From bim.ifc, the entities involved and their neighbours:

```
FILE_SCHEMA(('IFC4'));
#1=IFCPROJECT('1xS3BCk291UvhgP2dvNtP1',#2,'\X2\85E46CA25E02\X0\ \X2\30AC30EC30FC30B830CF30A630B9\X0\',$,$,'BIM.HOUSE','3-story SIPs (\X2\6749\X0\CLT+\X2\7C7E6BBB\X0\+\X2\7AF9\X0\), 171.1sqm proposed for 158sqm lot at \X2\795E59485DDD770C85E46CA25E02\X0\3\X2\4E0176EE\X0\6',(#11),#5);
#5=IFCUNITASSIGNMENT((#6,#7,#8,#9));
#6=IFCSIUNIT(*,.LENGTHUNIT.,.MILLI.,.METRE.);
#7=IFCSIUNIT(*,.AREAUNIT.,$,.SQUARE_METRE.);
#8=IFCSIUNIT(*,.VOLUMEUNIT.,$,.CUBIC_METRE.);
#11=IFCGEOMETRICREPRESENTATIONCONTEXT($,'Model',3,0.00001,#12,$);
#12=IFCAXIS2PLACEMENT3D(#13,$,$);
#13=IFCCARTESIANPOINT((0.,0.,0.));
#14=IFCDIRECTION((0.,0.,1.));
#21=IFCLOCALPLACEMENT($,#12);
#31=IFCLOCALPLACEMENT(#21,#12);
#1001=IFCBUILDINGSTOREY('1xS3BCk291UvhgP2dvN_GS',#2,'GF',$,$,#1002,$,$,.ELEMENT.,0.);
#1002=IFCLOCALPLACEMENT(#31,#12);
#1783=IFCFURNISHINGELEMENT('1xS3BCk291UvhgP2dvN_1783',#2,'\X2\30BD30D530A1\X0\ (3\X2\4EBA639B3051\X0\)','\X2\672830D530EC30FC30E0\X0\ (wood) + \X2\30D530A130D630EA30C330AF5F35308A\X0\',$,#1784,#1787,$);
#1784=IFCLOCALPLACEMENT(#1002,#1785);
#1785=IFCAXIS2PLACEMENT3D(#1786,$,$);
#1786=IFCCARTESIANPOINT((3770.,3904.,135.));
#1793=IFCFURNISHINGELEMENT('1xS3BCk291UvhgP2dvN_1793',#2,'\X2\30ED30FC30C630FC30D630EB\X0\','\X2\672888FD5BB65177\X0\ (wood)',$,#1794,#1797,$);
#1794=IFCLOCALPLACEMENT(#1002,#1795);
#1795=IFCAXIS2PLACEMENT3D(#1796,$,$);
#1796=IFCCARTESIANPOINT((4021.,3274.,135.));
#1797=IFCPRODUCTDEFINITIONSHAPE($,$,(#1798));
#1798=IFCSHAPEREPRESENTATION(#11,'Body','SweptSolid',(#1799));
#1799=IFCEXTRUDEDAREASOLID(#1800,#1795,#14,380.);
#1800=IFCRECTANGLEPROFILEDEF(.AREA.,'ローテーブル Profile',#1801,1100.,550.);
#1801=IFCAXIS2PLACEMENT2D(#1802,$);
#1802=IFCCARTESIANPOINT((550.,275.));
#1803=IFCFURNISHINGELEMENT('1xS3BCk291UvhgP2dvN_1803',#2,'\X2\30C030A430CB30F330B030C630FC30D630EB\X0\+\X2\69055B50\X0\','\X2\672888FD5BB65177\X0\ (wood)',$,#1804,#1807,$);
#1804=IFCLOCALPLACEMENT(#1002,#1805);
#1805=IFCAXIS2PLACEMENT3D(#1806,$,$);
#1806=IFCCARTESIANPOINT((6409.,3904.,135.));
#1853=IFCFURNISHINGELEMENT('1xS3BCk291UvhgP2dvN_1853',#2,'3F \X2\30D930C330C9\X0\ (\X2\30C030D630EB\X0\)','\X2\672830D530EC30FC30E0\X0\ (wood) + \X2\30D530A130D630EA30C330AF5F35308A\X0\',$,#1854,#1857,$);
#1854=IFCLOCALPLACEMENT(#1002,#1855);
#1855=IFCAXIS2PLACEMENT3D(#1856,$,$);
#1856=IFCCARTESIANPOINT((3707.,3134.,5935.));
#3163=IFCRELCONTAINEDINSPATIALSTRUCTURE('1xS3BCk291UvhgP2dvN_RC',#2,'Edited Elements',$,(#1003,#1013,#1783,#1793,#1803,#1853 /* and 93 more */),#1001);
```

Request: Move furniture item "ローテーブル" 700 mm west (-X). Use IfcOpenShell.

```python
import ifcopenshell
import ifcopenshell.api.geometry
import ifcopenshell.util.placement
import ifcopenshell.util.unit

model = ifcopenshell.open("bim.ifc")
unit_scale = ifcopenshell.util.unit.calculate_unit_scale(model)

item = model.by_id(1793)
matrix = ifcopenshell.util.placement.get_local_placement(item.ObjectPlacement)
matrix[0, 3] -= 0.7 / unit_scale
ifcopenshell.api.geometry.edit_object_placement(model, product=item, matrix=matrix, is_si=False)

print(ifcopenshell.util.placement.get_local_placement(item.ObjectPlacement).round(3) + 0.0)

model.write("bim_v2.ifc")
```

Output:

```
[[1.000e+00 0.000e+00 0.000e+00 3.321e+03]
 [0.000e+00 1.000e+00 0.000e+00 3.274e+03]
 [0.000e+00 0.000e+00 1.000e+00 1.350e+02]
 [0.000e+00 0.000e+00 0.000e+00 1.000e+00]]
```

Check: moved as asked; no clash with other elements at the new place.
